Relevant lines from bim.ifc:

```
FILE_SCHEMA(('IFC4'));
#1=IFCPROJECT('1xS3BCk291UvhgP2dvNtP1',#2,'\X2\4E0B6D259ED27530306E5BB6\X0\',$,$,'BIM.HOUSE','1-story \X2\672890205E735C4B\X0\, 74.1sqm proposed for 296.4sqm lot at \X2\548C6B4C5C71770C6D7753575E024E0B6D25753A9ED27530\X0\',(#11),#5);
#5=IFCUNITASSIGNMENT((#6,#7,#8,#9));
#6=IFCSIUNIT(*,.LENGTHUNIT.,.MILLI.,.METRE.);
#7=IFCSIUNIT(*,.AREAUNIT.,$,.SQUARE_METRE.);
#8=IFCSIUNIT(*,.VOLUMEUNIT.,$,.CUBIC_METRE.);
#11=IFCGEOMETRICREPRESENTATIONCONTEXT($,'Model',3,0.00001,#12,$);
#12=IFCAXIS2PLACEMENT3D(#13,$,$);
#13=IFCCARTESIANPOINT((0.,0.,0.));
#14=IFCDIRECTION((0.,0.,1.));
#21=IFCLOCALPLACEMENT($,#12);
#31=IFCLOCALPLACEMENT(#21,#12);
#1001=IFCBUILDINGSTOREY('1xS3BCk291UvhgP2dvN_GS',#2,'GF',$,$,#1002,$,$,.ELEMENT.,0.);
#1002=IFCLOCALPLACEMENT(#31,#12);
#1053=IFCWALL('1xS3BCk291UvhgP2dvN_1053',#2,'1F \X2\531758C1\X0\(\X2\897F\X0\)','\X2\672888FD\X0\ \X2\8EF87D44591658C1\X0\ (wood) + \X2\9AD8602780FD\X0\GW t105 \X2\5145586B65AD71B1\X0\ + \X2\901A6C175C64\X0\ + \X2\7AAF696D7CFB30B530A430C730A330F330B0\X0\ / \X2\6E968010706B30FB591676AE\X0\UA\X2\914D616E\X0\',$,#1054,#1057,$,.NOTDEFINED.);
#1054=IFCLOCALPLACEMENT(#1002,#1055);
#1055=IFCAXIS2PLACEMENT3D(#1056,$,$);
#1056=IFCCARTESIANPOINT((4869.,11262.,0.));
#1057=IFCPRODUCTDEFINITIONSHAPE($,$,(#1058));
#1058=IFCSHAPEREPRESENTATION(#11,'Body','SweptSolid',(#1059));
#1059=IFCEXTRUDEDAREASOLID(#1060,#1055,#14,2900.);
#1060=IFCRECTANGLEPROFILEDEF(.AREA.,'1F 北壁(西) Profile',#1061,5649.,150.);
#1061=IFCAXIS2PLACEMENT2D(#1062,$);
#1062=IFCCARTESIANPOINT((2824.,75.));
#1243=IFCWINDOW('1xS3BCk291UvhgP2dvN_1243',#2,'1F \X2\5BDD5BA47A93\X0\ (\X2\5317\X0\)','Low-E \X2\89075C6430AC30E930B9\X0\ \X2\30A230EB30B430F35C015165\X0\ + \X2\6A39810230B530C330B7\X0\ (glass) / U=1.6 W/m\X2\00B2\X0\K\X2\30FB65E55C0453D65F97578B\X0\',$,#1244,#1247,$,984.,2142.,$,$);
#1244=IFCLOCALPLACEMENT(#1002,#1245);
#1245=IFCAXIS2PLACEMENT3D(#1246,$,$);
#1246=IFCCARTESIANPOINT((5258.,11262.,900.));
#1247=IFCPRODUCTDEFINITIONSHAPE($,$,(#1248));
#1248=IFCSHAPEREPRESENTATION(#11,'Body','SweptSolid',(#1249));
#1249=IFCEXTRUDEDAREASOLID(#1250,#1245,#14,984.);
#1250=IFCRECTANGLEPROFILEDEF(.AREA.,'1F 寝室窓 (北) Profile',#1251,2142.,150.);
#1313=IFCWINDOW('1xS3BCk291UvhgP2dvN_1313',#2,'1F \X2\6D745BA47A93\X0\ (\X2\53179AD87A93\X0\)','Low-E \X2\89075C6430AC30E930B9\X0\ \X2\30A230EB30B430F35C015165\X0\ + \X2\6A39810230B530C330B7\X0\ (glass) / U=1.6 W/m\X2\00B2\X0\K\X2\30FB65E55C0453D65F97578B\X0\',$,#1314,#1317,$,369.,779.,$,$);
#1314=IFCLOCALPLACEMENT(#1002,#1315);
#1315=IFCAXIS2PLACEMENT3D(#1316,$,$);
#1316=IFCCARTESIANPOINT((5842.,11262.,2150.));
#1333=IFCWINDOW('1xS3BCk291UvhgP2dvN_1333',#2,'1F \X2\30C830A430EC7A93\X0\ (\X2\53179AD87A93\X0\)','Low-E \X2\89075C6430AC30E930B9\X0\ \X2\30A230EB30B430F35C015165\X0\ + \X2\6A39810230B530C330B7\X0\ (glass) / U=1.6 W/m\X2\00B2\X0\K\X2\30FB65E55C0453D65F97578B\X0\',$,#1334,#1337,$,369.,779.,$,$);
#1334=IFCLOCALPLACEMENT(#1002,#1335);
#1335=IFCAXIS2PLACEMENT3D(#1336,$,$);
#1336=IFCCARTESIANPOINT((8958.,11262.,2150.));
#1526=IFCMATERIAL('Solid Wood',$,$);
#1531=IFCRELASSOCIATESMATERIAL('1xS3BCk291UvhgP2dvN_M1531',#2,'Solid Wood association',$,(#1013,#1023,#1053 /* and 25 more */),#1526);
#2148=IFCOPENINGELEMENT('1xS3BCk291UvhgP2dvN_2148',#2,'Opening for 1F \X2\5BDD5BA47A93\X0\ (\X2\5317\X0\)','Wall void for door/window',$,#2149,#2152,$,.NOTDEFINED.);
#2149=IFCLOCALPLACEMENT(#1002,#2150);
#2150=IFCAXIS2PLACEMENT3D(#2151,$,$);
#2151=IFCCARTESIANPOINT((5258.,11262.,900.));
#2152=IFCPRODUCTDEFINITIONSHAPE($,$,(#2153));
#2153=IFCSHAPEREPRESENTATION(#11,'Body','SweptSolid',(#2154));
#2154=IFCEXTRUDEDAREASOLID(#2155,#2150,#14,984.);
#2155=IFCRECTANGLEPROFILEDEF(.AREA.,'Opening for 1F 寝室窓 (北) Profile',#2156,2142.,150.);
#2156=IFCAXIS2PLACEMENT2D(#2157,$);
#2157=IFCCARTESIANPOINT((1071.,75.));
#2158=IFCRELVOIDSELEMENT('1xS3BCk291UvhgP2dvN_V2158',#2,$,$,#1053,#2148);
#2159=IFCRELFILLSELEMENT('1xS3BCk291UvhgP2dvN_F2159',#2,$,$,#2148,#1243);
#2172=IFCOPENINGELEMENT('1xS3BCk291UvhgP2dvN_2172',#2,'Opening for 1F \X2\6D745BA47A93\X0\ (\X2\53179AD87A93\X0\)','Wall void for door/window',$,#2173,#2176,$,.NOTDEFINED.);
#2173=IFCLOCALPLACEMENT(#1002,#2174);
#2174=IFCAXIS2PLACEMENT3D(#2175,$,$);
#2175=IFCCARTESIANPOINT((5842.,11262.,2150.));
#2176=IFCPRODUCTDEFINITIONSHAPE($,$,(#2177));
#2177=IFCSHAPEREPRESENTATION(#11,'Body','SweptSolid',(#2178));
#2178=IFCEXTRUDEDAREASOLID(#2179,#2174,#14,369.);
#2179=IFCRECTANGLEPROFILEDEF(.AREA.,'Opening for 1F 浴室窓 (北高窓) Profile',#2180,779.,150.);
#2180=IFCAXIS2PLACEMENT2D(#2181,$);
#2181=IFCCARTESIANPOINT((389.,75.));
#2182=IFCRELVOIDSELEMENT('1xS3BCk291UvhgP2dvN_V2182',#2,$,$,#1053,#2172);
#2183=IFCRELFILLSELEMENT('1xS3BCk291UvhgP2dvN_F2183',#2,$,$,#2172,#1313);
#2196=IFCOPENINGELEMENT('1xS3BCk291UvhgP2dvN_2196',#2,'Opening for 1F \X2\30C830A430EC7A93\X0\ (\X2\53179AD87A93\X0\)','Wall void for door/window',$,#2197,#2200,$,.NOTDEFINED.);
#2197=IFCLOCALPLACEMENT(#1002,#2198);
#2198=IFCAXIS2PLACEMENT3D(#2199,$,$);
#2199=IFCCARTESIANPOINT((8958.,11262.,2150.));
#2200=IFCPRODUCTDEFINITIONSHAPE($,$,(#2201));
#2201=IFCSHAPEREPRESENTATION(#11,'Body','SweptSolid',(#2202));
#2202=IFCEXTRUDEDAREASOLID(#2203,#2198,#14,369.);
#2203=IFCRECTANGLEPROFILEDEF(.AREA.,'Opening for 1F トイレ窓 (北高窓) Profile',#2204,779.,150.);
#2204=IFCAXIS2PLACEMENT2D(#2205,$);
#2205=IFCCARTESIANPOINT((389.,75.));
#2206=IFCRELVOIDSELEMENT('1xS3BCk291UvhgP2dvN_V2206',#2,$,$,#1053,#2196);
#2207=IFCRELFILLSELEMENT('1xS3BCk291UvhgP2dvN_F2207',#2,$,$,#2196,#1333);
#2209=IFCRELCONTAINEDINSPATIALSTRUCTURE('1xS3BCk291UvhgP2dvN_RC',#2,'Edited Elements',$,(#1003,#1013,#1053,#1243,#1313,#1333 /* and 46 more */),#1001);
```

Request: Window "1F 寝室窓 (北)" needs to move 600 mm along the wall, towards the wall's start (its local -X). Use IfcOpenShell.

```python
import ifcopenshell
import ifcopenshell.api.geometry
import ifcopenshell.util.placement

model = ifcopenshell.open("bim.ifc")

window = model.by_id(1243)
opening = window.FillsVoids[0].RelatingOpeningElement
wall = opening.VoidsElements[0].RelatingBuildingElement

wall_matrix = ifcopenshell.util.placement.get_local_placement(wall.ObjectPlacement)
shift = wall_matrix[:3, 0] * -600.0
before = ifcopenshell.util.placement.get_local_placement(window.ObjectPlacement)[:3, 3].copy()

# The window is not placed relative to its opening, so move both.
for product in (opening, window):
    matrix = ifcopenshell.util.placement.get_local_placement(product.ObjectPlacement)
    matrix[:3, 3] += shift
    ifcopenshell.api.geometry.edit_object_placement(model, product=product, matrix=matrix, is_si=False)

after = ifcopenshell.util.placement.get_local_placement(window.ObjectPlacement)[:3, 3]
print("window moved by", (after - before).round(3) + 0.0)

model.write("bim_v2.ifc")
```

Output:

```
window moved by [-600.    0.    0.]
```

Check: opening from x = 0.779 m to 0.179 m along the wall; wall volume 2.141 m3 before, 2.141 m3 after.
